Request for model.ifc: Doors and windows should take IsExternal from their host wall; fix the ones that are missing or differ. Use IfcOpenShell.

First a look at what the model holds.

```python
import ifcopenshell
import ifcopenshell.util.element

model = ifcopenshell.open("model.ifc")
print(model.schema)
seen = {}
for e in model.by_type("IfcDoor") + model.by_type("IfcWindow"):
    if not e.FillsVoids:
        continue
    host = e.FillsVoids[0].RelatingOpeningElement.VoidsElements[0].RelatingBuildingElement
    own = ifcopenshell.util.element.get_pset(e, f"Pset_{e.is_a()[3:].removesuffix('StandardCase')}Common", "IsExternal")
    wall = ifcopenshell.util.element.get_pset(host, "Pset_WallCommon", "IsExternal")
    seen[e.is_a(), own, wall] = seen.get((e.is_a(), own, wall), 0) + 1
for (cls, own, wall), count in sorted(seen.items(), key=str):
    print(count, cls, "IsExternal:", own, "| host wall:", wall)
```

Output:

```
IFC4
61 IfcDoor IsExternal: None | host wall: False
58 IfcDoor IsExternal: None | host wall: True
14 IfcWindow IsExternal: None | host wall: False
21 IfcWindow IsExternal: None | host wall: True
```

```python
import ifcopenshell
import ifcopenshell.api.pset
import ifcopenshell.util.element

model = ifcopenshell.open("model.ifc")

count = 0
for ifc_class, pset_name in (("IfcDoor", "Pset_DoorCommon"), ("IfcWindow", "Pset_WindowCommon")):
    for e in model.by_type(ifc_class):
        if not e.FillsVoids:
            continue
        host = e.FillsVoids[0].RelatingOpeningElement.VoidsElements[0].RelatingBuildingElement
        external = ifcopenshell.util.element.get_pset(host, "Pset_WallCommon", "IsExternal")
        if external is None or ifcopenshell.util.element.get_pset(e, pset_name, "IsExternal") == external:
            continue
        pset = ifcopenshell.api.pset.add_pset(model, product=e, name=pset_name)
        ifcopenshell.api.pset.edit_pset(model, pset=pset, properties={"IsExternal": external})
        count += 1

print(count, "updated")

model.write("model_edited.ifc")
```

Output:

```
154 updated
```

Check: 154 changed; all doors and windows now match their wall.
